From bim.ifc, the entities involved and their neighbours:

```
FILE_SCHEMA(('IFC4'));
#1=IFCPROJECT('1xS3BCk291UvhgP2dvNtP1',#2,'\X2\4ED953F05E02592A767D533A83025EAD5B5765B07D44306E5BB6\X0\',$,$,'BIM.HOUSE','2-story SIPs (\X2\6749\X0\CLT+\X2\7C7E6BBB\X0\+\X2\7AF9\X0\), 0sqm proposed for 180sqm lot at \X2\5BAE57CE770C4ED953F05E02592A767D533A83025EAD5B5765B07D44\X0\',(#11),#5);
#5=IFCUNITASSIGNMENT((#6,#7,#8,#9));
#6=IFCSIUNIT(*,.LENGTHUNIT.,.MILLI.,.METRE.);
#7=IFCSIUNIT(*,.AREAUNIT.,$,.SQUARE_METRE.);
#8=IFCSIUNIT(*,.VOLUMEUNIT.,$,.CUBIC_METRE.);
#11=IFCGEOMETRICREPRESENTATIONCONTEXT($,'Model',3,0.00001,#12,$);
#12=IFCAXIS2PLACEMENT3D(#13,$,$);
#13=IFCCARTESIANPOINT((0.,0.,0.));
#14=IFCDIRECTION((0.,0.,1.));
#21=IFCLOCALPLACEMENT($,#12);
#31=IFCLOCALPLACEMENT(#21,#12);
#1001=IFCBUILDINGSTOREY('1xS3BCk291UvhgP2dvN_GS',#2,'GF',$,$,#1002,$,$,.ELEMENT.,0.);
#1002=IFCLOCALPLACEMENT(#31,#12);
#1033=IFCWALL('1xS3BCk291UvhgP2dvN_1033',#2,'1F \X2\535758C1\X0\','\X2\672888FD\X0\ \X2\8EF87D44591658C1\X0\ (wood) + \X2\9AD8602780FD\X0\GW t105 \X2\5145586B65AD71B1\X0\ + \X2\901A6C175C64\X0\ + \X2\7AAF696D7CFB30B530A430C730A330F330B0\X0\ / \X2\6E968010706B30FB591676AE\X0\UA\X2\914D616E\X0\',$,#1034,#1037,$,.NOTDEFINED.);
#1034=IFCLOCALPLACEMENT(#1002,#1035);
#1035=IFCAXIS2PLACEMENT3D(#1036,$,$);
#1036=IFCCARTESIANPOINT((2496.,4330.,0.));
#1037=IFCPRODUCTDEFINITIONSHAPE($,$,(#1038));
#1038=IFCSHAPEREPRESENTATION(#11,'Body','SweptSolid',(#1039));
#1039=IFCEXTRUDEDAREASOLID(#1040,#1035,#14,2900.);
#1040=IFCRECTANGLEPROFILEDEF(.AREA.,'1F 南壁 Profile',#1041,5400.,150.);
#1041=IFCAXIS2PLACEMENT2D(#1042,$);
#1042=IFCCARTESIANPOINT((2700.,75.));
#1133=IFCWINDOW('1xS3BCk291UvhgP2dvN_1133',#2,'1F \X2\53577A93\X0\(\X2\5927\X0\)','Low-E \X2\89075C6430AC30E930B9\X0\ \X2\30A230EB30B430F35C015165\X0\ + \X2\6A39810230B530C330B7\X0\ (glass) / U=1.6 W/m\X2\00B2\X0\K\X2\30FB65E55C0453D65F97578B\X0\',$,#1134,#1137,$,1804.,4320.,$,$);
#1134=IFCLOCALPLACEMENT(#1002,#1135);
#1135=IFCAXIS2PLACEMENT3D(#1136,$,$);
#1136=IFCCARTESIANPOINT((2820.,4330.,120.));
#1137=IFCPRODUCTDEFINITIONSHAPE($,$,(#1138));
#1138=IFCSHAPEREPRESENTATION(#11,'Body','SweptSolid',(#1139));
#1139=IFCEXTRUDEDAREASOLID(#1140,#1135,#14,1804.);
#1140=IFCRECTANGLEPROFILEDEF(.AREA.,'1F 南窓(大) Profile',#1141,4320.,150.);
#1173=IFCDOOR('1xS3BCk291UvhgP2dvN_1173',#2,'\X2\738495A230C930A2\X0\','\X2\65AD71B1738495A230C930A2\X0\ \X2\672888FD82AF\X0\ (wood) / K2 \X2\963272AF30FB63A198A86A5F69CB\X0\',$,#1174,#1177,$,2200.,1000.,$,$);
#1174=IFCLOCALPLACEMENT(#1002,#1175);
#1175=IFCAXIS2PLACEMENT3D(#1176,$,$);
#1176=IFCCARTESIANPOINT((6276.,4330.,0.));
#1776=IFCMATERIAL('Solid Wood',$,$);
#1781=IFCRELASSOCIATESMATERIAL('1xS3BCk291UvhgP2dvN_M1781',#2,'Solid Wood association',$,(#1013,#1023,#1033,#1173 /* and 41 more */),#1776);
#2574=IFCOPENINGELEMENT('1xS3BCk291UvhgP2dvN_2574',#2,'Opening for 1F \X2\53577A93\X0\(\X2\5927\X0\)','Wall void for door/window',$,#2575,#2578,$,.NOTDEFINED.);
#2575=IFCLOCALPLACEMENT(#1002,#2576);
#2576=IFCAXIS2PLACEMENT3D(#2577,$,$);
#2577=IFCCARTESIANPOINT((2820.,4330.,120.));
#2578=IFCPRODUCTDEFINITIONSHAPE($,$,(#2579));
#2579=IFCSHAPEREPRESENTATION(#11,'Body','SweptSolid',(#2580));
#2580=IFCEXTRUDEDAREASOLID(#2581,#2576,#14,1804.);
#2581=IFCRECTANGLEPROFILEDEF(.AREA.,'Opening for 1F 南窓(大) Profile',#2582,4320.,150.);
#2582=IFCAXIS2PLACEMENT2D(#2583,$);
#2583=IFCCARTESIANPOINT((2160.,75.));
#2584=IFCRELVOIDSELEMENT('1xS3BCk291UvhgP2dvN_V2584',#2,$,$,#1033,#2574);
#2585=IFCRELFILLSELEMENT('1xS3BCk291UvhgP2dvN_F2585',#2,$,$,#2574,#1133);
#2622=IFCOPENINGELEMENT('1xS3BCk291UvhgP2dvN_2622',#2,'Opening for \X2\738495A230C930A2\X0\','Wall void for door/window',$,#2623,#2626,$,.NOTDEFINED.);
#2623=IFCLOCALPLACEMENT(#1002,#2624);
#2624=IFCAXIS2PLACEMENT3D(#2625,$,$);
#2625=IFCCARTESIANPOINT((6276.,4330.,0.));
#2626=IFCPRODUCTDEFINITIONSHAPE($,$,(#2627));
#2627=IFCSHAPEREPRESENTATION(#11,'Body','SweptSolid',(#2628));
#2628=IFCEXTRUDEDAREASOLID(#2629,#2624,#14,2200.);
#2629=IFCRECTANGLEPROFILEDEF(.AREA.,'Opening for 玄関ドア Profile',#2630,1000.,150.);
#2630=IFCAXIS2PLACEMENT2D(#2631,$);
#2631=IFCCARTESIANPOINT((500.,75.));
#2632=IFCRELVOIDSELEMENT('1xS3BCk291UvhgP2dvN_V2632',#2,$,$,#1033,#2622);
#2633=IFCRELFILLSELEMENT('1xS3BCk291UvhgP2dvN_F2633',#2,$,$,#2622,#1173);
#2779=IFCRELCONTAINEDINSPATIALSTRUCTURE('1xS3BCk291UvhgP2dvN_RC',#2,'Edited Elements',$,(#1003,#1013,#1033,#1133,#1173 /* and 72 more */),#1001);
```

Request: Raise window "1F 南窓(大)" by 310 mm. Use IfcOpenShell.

```python
import numpy as np
import ifcopenshell
import ifcopenshell.api.geometry
import ifcopenshell.util.placement
import ifcopenshell.util.unit

model = ifcopenshell.open("bim.ifc")
unit_scale = ifcopenshell.util.unit.calculate_unit_scale(model)

window = model.by_guid("1xS3BCk291UvhgP2dvN_1133")
opening = window.FillsVoids[0].RelatingOpeningElement
dz = 310.0

shift = np.array([0.0, 0.0, dz])
# The window is not placed relative to its opening, so move both.
for product in (opening, window):
    matrix = ifcopenshell.util.placement.get_local_placement(product.ObjectPlacement)
    matrix[:3, 3] += shift
    ifcopenshell.api.geometry.edit_object_placement(model, product=product, matrix=matrix, is_si=False)

print(f"moved by {dz * unit_scale:+.3f} m")

model.write("bim_v2.ifc")
```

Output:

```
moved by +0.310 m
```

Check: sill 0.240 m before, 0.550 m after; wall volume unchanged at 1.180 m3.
